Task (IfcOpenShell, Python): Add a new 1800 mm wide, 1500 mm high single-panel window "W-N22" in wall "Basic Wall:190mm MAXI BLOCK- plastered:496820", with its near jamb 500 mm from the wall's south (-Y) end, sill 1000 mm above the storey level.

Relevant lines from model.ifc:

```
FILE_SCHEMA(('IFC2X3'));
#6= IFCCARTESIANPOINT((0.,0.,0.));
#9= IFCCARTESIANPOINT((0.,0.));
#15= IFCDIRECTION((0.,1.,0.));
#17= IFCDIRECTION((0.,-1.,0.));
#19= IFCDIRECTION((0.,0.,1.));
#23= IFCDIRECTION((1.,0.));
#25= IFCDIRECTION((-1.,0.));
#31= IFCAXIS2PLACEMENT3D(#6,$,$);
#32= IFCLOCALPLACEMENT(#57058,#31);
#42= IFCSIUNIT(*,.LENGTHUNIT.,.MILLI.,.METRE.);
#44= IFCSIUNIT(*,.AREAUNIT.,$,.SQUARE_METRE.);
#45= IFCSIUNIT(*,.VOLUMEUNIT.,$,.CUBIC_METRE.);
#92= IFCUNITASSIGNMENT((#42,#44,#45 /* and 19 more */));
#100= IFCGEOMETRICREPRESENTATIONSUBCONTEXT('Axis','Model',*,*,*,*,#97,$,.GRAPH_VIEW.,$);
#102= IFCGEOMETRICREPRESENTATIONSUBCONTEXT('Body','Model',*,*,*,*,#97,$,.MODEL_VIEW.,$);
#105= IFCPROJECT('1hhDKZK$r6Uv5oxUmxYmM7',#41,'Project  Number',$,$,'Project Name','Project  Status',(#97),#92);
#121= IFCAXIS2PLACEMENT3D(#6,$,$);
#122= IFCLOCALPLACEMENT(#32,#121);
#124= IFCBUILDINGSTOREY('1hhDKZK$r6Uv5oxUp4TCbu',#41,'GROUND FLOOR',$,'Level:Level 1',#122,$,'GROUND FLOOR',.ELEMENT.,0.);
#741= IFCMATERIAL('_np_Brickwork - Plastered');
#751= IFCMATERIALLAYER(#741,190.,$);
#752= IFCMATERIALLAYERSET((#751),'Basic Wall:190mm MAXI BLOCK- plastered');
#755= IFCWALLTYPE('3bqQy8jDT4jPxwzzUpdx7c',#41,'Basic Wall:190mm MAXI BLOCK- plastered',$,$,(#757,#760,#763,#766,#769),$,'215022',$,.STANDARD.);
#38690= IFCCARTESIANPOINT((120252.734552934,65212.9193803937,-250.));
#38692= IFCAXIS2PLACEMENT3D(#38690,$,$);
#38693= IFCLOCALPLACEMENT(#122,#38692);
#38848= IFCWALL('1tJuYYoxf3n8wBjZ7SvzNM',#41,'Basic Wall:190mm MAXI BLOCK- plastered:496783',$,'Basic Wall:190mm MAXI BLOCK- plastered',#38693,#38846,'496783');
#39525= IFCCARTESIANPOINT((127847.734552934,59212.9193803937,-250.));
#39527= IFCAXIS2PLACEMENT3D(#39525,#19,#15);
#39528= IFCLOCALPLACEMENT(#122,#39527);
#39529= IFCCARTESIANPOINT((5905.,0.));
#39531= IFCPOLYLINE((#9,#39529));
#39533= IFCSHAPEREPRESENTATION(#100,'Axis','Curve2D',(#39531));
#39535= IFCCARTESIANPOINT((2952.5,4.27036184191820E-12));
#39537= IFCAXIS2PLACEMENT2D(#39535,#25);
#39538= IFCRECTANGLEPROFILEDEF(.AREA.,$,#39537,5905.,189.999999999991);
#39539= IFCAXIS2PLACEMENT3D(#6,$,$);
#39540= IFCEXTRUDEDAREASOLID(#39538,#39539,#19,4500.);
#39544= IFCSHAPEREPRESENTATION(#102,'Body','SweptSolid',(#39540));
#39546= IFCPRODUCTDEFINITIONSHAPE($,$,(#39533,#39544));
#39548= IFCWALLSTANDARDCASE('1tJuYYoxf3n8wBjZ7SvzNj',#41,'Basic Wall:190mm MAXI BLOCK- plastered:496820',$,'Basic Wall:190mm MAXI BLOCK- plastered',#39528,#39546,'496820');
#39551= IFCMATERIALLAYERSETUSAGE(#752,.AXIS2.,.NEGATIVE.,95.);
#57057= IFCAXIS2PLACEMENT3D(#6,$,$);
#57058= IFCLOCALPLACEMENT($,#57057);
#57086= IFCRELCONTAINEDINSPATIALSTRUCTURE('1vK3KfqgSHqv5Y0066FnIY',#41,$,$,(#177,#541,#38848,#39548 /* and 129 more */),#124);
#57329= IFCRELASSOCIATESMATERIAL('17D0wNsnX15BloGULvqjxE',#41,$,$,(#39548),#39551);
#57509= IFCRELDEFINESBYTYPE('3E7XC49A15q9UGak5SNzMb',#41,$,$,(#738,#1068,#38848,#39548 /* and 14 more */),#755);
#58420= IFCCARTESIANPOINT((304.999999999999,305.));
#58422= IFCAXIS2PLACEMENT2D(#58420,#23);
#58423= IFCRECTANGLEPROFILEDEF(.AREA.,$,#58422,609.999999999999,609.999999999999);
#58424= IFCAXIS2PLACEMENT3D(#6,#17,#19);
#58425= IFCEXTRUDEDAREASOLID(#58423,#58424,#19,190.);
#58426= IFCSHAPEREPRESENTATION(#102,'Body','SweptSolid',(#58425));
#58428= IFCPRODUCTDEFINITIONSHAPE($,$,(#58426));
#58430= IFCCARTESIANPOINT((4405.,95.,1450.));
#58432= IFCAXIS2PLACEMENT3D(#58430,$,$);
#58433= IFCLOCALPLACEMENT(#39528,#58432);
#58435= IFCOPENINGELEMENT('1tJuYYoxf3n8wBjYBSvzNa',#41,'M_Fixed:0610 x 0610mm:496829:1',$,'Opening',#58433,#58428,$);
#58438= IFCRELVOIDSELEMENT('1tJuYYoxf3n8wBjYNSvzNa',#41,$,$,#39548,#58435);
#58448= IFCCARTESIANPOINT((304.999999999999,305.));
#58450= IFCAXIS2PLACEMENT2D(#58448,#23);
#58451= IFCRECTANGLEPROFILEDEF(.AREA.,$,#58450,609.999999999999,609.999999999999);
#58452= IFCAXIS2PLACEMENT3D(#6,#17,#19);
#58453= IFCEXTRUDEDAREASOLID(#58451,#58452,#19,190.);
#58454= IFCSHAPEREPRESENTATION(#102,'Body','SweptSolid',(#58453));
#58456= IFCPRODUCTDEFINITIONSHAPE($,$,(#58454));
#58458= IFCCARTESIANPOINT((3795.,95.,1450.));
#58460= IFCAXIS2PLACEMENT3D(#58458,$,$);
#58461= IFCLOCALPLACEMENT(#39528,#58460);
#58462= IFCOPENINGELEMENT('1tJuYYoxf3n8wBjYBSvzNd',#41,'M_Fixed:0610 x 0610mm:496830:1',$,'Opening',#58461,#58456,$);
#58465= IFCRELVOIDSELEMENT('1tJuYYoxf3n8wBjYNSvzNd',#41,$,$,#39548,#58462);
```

```python
import numpy as np
import ifcopenshell
import ifcopenshell.api.feature
import ifcopenshell.api.geometry
import ifcopenshell.api.root
import ifcopenshell.api.spatial
import ifcopenshell.api.type
import ifcopenshell.geom
import ifcopenshell.util.element
import ifcopenshell.util.placement
import ifcopenshell.util.representation
import ifcopenshell.util.shape
import ifcopenshell.util.unit

model = ifcopenshell.open("model.ifc")
unit_scale = ifcopenshell.util.unit.calculate_unit_scale(model)
settings = ifcopenshell.geom.settings()


def volume(element):
    """Net volume in cubic metres, openings subtracted."""
    shape = ifcopenshell.geom.create_shape(settings, element)
    return ifcopenshell.util.shape.get_volume(shape.geometry)


wall = model.by_guid("1tJuYYoxf3n8wBjZ7SvzNj")
storey = ifcopenshell.util.element.get_container(wall, ifc_class="IfcBuildingStorey")
context = ifcopenshell.util.representation.get_context(model, "Model", "Body", "MODEL_VIEW")
before = volume(wall)

width, height, from_end, sill = 1.8, 1.5, 0.5, 1  # metres

# The wall runs along its own X axis, and the end named is its -X end.
wall_shape = ifcopenshell.geom.create_shape(settings, wall)
x, y, z = ifcopenshell.util.shape.get_vertices(wall_shape.geometry).T
start = x.min() + from_end
face, thickness = float(y.min()), float(y.max() - y.min())
wall_matrix = ifcopenshell.util.placement.get_local_placement(wall.ObjectPlacement)
level = ifcopenshell.util.placement.get_local_placement(storey.ObjectPlacement)[2, 3]


def in_wall(x, y):
    """Placement at x, y metres in the wall's axes, at sill height."""
    matrix = wall_matrix.copy()
    matrix[:, 3] = wall_matrix @ np.array([x / unit_scale, y / unit_scale, 0.0, 1.0])
    matrix[2, 3] = level + sill / unit_scale
    return matrix


# Opening: a box that overshoots both wall faces by 50 mm.
opening = ifcopenshell.api.root.create_entity(model, ifc_class="IfcOpeningElement")
box = ifcopenshell.api.geometry.add_wall_representation(
    model, context=context, length=width, height=height, thickness=thickness + 0.1
)
ifcopenshell.api.geometry.assign_representation(model, product=opening, representation=box)
ifcopenshell.api.geometry.edit_object_placement(model, product=opening, matrix=in_wall(start, face - 0.05), is_si=False)
ifcopenshell.api.feature.add_feature(model, feature=opening, element=wall)

window = ifcopenshell.api.root.create_entity(model, ifc_class="IfcWindow", name="W-N22")
window.OverallWidth, window.OverallHeight = width / unit_scale, height / unit_scale
body = ifcopenshell.api.geometry.add_window_representation(
    model,
    context=context,
    overall_width=window.OverallWidth,
    overall_height=window.OverallHeight,
    partition_type="SINGLE_PANEL",
)
ifcopenshell.api.geometry.assign_representation(model, product=window, representation=body)
ifcopenshell.api.spatial.assign_container(model, products=[window], relating_structure=storey)
fills = ifcopenshell.api.feature.add_filling(model, opening=opening, element=window)
fills.OwnerHistory = window.OwnerHistory  # required in IFC2X3

# IFC2X3 keeps the operation on the window style.
style = ifcopenshell.api.root.create_entity(model, ifc_class="IfcWindowStyle", name="W-N22")
style.OperationType, style.ConstructionType = "SINGLE_PANEL", "NOTDEFINED"
style.ParameterTakesPrecedence = style.Sizeable = False
ifcopenshell.api.type.assign_type(model, related_objects=[window], relating_type=style)

# Centre the window in the wall's thickness.
ifcopenshell.api.geometry.edit_object_placement(model, product=window, matrix=in_wall(start, face), is_si=False)
window_shape = ifcopenshell.geom.create_shape(settings, window)
depth = ifcopenshell.util.shape.get_vertices(window_shape.geometry)[:, 1]
offset = face + thickness / 2 - (depth.min() + depth.max()) / 2
ifcopenshell.api.geometry.edit_object_placement(model, product=window, matrix=in_wall(start, offset), is_si=False)

after = volume(wall)

print(f"wall volume {before:.3f} -> {after:.3f} m3")

model.write("model_v2.ifc")
```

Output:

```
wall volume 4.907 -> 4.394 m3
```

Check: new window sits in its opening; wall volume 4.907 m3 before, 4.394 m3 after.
